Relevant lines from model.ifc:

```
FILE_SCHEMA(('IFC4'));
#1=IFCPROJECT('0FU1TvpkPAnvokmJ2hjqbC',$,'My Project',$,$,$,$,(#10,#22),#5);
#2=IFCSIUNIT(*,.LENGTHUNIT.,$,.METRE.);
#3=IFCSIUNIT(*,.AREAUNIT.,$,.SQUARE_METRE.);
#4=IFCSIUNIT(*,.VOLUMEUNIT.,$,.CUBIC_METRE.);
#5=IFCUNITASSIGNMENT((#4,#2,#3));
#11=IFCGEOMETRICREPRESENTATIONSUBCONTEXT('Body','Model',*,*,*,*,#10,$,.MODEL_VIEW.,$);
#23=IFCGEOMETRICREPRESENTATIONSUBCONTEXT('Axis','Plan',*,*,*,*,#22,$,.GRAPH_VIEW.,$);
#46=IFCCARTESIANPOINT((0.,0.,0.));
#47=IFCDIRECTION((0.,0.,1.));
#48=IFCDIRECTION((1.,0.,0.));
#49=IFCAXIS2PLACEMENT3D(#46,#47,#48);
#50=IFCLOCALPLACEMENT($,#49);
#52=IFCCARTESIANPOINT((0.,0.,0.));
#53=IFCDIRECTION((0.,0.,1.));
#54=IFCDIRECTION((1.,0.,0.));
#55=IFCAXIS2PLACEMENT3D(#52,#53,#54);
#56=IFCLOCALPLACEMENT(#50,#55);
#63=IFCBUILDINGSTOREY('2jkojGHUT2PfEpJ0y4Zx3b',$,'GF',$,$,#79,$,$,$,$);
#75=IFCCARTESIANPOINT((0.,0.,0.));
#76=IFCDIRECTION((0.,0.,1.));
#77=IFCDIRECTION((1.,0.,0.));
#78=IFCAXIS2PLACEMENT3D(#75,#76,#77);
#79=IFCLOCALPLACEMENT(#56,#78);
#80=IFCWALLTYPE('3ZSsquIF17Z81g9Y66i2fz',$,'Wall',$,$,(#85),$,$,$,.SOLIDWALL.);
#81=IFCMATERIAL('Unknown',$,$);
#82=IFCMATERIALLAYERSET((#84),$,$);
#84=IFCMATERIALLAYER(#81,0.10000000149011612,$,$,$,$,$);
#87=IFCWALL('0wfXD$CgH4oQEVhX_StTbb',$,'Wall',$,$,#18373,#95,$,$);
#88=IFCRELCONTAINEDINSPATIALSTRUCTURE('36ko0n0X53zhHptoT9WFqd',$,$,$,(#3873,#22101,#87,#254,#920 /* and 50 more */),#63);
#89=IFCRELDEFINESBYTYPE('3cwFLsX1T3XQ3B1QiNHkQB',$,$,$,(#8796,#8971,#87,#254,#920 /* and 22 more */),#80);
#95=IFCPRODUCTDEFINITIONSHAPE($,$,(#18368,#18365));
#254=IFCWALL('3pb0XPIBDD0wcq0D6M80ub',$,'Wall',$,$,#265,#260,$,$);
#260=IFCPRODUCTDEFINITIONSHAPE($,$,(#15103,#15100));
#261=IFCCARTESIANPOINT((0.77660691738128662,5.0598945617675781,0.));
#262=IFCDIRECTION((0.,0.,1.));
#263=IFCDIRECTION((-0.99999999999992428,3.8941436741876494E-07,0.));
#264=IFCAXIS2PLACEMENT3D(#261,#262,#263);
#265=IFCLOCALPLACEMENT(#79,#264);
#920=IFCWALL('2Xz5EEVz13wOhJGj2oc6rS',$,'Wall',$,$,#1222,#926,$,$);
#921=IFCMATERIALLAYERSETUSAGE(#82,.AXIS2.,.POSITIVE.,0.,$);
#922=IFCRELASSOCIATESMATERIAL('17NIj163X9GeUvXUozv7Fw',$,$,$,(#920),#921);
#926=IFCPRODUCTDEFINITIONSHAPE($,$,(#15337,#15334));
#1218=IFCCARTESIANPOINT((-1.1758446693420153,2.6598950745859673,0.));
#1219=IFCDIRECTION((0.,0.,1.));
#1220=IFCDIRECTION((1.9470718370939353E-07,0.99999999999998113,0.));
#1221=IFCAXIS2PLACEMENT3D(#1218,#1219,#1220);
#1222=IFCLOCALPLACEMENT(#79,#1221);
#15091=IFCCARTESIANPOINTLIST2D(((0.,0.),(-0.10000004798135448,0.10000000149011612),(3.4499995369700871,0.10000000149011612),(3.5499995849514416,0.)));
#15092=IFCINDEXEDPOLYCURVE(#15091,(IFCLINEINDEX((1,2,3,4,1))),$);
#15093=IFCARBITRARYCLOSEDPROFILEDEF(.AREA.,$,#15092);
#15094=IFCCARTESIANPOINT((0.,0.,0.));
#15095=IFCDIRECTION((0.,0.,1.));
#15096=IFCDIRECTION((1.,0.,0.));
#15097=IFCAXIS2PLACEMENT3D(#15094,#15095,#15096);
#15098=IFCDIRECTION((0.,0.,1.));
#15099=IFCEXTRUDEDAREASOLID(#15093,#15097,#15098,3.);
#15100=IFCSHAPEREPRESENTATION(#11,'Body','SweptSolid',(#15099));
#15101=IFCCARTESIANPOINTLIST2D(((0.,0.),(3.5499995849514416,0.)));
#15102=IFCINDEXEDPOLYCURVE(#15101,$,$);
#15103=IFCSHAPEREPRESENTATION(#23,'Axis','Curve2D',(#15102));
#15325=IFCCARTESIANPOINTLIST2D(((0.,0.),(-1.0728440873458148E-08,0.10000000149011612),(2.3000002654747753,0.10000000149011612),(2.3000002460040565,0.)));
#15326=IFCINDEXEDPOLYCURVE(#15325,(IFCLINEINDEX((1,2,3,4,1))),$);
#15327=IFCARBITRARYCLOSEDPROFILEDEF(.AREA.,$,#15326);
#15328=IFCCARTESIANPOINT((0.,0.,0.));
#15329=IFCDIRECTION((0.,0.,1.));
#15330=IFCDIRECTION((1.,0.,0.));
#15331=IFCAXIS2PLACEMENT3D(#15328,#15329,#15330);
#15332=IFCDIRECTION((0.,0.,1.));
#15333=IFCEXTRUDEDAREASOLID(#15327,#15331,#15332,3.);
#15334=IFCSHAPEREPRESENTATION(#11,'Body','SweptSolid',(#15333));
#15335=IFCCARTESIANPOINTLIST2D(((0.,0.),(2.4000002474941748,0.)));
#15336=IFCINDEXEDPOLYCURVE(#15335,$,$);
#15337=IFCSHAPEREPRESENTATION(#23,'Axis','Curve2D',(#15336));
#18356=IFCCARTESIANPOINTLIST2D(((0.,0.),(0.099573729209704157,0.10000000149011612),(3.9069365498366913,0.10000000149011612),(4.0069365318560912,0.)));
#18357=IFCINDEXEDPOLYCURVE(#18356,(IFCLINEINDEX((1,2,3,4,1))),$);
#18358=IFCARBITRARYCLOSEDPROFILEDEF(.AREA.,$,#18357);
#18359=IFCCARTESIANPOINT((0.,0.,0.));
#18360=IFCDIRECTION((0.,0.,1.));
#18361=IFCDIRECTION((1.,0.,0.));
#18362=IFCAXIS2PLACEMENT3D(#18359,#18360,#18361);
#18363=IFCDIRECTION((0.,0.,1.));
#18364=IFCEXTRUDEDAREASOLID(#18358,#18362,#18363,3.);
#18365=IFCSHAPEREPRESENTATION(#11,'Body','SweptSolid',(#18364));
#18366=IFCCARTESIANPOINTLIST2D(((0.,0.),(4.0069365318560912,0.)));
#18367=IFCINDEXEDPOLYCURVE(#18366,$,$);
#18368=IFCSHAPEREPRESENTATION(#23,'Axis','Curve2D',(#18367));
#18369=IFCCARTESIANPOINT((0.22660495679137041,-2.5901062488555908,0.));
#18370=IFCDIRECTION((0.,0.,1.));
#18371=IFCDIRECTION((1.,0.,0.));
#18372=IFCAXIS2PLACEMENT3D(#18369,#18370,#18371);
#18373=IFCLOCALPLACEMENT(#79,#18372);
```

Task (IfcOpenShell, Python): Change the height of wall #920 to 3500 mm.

```python
import ifcopenshell
import ifcopenshell.geom
import ifcopenshell.util.representation
import ifcopenshell.util.shape
import ifcopenshell.util.unit

model = ifcopenshell.open("model.ifc")
unit_scale = ifcopenshell.util.unit.calculate_unit_scale(model)
settings = ifcopenshell.geom.settings()


def volume(element):
    """Net volume in cubic metres, openings subtracted."""
    shape = ifcopenshell.geom.create_shape(settings, element)
    return ifcopenshell.util.shape.get_volume(shape.geometry)


wall = model.by_guid("2Xz5EEVz13wOhJGj2oc6rS")
before = volume(wall)

body = ifcopenshell.util.representation.get_representation(wall, "Model", "Body")
solid = body.Items[0]
old_height = solid.Depth
solid.Depth = 3.5 / unit_scale
after = volume(wall)

print(f"height {old_height:g} -> {solid.Depth:g}, volume {before:.3f} -> {after:.3f} m3")

model.write("model_v2.ifc")
```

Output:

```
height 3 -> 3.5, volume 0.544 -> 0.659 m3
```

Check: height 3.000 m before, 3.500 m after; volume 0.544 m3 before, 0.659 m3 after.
